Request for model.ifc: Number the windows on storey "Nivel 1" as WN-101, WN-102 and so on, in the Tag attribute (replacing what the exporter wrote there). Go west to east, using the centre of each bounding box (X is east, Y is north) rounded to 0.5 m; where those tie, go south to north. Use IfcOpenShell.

First a look at what the model holds.

```python
import ifcopenshell
import ifcopenshell.util.element
import ifcopenshell.util.placement

model = ifcopenshell.open("model.ifc")
print(model.schema)
storey = next(s for s in model.by_type("IfcBuildingStorey") if s.Name == "Nivel 1")
windows = [e for e in ifcopenshell.util.element.get_decomposition(storey) if e.is_a("IfcWindow")]
for e in sorted(windows, key=lambda e: e.id()):
    origin = ifcopenshell.util.placement.get_local_placement(e.ObjectPlacement)[:3, 3]
    print(e.id(), e.Tag, e.Name, origin.round(2) + 0.0, sep=" | ")
```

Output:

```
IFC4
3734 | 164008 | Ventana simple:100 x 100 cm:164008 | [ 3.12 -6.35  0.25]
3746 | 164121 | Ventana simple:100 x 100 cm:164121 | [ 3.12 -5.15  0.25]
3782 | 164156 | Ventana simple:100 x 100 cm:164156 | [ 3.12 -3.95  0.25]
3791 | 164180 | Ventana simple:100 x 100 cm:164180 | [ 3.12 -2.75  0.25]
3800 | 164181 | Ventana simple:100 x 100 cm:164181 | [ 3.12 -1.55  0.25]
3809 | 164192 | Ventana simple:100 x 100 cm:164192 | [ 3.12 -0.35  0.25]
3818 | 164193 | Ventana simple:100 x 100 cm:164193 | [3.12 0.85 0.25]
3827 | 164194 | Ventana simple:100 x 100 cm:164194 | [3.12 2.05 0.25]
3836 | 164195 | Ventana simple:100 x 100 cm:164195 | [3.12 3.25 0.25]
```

```python
import ifcopenshell
import ifcopenshell.geom
import ifcopenshell.util.element
import ifcopenshell.util.shape

model = ifcopenshell.open("model.ifc")
settings = ifcopenshell.geom.settings()
settings.set("use-world-coords", True)


def centre(element):
    shape = ifcopenshell.geom.create_shape(settings, element)
    return ifcopenshell.util.shape.get_bbox_centroid(shape.geometry)


storey = next(s for s in model.by_type("IfcBuildingStorey") if s.Name == "Nivel 1")
windows = [e for e in ifcopenshell.util.element.get_decomposition(storey) if e.is_a("IfcWindow")]

# Insertion points can sit at a corner or the storey origin, so sort by the geometry (in metres).
centres = {e: centre(e) for e in windows}
windows.sort(key=lambda e: (round(centres[e][0] / 0.5), centres[e][1]))

for i, e in enumerate(windows, start=1):
    number = f"WN-1{i:02d}"
    e.Tag = number
    print(e.id(), number)

model.write("model_v2.ifc")
```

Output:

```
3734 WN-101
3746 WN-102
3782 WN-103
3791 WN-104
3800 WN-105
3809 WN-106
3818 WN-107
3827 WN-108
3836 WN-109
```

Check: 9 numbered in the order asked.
